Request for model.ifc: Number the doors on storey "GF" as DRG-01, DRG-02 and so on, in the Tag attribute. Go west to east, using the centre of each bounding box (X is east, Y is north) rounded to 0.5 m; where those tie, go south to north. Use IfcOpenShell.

First a look at what the model holds.

```python
import ifcopenshell
import ifcopenshell.util.element
import ifcopenshell.util.placement

model = ifcopenshell.open("model.ifc")
print(model.schema)
storey = next(s for s in model.by_type("IfcBuildingStorey") if s.Name == "GF")
doors = [e for e in ifcopenshell.util.element.get_decomposition(storey) if e.is_a("IfcDoor")]
for e in sorted(doors, key=lambda e: e.id()):
    origin = ifcopenshell.util.placement.get_local_placement(e.ObjectPlacement)[:3, 3]
    print(e.id(), e.Tag, e.Name, origin.round(2) + 0.0, sep=" | ")
```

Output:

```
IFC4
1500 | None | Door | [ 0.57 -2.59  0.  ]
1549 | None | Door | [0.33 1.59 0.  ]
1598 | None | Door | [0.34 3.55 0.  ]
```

```python
import ifcopenshell
import ifcopenshell.geom
import ifcopenshell.util.element
import ifcopenshell.util.shape

model = ifcopenshell.open("model.ifc")
settings = ifcopenshell.geom.settings()
settings.set("use-world-coords", True)


def centre(element):
    shape = ifcopenshell.geom.create_shape(settings, element)
    return ifcopenshell.util.shape.get_bbox_centroid(shape.geometry)


storey = next(s for s in model.by_type("IfcBuildingStorey") if s.Name == "GF")
doors = [e for e in ifcopenshell.util.element.get_decomposition(storey) if e.is_a("IfcDoor")]

# Insertion points can sit at a corner or the storey origin, so sort by the geometry (in metres).
centres = {e: centre(e) for e in doors}
doors.sort(key=lambda e: (round(centres[e][0] / 0.5), centres[e][1]))

for i, e in enumerate(doors, start=1):
    number = f"DRG-{i:02d}"
    e.Tag = number
    print(e.id(), number)

model.write("model_rev.ifc")
```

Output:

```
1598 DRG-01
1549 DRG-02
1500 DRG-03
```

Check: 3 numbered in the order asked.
